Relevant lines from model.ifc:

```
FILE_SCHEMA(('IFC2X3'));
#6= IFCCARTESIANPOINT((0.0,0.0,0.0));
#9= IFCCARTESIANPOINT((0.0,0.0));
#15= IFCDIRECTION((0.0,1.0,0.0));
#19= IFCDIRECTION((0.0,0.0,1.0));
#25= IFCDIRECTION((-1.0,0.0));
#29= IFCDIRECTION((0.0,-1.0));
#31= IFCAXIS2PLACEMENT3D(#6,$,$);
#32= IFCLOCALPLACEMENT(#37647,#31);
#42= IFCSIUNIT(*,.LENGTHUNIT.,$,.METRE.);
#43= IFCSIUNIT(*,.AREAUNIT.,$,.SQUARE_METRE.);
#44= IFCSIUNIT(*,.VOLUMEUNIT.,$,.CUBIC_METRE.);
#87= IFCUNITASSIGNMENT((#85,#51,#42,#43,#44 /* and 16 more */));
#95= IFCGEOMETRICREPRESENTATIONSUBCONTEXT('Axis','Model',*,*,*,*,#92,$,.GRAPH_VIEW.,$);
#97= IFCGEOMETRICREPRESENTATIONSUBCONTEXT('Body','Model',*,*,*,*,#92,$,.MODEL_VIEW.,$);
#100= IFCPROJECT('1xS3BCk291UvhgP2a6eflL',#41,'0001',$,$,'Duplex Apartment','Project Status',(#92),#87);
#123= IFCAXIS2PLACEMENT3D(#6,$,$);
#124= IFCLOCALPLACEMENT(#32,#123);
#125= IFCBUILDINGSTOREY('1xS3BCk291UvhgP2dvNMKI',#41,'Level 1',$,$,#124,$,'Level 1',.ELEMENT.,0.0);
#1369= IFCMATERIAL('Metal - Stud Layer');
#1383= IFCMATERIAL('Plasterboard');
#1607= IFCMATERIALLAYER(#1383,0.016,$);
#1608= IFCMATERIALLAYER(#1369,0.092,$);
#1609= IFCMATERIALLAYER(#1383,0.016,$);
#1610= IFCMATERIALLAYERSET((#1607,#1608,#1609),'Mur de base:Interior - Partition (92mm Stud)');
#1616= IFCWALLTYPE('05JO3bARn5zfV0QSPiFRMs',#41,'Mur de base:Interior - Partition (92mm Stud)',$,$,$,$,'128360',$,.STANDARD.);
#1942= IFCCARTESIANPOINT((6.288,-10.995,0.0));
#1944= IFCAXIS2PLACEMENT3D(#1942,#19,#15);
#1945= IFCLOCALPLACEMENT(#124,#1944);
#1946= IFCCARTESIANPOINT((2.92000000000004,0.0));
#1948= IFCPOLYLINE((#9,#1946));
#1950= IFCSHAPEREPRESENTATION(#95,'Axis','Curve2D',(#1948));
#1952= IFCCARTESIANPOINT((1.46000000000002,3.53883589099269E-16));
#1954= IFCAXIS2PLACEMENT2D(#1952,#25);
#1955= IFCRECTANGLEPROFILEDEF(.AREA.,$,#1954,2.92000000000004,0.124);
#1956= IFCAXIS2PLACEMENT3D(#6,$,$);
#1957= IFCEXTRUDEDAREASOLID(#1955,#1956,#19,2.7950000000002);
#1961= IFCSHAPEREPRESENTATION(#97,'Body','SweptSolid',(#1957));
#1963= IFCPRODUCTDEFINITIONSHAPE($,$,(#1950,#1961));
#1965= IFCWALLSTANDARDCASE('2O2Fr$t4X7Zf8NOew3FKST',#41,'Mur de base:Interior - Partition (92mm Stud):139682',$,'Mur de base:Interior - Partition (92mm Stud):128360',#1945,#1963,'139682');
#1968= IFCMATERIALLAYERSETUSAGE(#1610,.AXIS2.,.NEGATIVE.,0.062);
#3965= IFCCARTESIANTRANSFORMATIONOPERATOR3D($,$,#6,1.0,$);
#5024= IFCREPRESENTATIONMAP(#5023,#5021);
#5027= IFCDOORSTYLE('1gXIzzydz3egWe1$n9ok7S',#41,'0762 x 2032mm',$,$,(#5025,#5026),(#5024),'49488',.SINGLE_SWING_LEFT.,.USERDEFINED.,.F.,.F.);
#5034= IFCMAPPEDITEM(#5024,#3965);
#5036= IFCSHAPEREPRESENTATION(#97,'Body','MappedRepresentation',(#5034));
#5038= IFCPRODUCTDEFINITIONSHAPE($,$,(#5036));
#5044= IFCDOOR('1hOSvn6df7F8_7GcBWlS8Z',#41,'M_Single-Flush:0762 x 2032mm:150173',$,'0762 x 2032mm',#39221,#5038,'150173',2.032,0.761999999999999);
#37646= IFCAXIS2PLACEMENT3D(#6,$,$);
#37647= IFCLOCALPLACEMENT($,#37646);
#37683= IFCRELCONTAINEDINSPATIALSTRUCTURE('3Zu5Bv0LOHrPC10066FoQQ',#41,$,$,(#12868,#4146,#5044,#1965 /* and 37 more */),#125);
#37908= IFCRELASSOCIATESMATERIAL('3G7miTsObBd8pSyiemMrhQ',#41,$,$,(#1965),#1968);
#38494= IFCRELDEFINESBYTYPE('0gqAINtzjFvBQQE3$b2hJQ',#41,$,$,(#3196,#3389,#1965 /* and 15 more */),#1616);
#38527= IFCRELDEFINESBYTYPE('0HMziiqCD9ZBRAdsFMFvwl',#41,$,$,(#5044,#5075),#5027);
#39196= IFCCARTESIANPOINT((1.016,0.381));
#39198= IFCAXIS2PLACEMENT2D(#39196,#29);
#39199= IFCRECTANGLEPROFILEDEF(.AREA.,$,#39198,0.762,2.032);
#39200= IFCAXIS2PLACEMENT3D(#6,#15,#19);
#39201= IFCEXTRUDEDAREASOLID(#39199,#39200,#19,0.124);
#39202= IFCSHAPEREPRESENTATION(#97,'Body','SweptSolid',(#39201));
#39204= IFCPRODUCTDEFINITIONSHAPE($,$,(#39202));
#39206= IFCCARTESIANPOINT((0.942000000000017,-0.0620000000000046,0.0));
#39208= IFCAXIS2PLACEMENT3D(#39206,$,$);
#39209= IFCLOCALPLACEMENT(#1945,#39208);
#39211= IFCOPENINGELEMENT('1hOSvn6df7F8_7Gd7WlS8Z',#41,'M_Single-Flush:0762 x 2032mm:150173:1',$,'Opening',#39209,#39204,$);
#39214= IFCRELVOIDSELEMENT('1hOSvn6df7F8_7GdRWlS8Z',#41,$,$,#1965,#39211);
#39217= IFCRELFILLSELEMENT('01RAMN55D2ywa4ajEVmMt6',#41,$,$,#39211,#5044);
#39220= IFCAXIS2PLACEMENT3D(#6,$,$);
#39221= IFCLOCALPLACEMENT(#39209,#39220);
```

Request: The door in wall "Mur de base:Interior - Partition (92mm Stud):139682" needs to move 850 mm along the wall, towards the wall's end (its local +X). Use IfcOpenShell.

```python
import ifcopenshell
import ifcopenshell.api.geometry
import ifcopenshell.util.placement
import ifcopenshell.util.unit

model = ifcopenshell.open("model.ifc")
unit_scale = ifcopenshell.util.unit.calculate_unit_scale(model)

door = model.by_guid("1hOSvn6df7F8_7GcBWlS8Z")
opening = door.FillsVoids[0].RelatingOpeningElement
wall = opening.VoidsElements[0].RelatingBuildingElement

wall_matrix = ifcopenshell.util.placement.get_local_placement(wall.ObjectPlacement)
shift = wall_matrix[:3, 0] * 0.85 / unit_scale
before = ifcopenshell.util.placement.get_local_placement(door.ObjectPlacement)[:3, 3].copy()

# The door is placed relative to its opening, so it follows when the opening moves.
matrix = ifcopenshell.util.placement.get_local_placement(opening.ObjectPlacement)
matrix[:3, 3] += shift
ifcopenshell.api.geometry.edit_object_placement(
    model, product=opening, matrix=matrix, is_si=False, should_transform_children=True
)

after = ifcopenshell.util.placement.get_local_placement(door.ObjectPlacement)[:3, 3]
print("door moved by", (after - before).round(3) + 0.0)

model.write("model_rev.ifc")
```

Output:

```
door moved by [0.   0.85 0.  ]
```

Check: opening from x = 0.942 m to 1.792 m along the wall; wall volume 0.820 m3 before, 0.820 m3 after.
